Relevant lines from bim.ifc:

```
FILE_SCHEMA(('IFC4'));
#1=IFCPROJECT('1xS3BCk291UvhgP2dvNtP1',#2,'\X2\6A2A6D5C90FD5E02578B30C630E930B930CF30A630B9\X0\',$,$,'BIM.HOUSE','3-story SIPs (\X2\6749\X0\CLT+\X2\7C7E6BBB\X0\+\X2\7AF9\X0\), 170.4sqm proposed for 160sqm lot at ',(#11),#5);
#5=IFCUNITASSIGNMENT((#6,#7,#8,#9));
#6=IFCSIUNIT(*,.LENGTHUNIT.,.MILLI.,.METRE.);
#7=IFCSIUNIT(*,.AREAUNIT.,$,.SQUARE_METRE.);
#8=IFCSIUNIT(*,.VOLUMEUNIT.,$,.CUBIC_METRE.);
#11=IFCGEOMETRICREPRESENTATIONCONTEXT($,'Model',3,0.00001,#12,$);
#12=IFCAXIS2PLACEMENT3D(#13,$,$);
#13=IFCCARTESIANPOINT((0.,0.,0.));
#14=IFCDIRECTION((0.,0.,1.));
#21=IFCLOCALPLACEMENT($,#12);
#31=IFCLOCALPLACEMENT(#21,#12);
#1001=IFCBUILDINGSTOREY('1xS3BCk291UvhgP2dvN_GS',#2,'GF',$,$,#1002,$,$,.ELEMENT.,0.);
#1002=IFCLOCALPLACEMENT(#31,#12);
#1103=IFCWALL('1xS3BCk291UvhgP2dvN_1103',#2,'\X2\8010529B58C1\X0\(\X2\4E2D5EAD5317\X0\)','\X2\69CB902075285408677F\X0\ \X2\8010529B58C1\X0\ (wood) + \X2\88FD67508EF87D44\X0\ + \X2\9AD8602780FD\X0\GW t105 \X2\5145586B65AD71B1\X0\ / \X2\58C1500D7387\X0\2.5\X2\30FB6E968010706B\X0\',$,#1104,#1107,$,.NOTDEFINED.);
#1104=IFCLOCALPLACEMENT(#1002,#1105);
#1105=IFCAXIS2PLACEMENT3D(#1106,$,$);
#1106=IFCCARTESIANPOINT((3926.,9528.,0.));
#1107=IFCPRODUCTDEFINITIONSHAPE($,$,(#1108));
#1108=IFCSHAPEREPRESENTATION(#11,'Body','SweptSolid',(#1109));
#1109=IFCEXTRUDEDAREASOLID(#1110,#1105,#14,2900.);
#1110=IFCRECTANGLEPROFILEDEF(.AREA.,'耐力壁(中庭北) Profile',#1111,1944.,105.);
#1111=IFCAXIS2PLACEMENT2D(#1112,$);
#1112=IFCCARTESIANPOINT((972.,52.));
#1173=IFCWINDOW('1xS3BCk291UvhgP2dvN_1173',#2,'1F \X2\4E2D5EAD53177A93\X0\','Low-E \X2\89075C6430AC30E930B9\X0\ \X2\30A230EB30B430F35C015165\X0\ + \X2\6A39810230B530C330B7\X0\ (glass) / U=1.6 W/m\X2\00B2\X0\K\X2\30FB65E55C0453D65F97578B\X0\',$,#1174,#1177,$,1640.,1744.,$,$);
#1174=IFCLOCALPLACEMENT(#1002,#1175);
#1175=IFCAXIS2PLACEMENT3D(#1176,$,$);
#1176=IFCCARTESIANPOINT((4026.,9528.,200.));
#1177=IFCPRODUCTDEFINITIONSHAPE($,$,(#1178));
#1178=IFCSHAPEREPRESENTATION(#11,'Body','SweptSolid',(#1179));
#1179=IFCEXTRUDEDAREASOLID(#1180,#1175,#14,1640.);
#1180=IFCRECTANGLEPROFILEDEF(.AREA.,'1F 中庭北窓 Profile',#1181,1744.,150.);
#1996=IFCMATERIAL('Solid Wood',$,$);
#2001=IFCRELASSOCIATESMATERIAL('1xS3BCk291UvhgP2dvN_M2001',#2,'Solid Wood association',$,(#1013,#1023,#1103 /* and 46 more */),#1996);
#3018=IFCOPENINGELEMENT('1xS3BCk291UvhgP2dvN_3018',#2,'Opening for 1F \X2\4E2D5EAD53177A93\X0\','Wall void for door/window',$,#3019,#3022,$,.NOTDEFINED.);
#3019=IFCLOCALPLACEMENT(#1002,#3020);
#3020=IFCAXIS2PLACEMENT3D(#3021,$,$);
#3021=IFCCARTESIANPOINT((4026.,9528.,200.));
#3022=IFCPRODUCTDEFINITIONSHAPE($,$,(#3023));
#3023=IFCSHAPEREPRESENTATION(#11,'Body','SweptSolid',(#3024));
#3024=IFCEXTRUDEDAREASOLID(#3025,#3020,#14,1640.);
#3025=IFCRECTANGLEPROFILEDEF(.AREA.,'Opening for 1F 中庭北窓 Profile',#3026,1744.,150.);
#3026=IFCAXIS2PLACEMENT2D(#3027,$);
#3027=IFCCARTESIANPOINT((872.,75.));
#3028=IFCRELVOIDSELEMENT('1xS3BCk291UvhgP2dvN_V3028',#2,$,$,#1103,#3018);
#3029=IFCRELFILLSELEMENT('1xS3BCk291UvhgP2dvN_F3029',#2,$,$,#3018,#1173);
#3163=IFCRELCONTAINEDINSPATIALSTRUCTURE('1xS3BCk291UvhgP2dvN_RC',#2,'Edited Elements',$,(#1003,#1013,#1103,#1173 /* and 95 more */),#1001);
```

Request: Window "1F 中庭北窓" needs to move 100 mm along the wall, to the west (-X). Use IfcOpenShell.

```python
import ifcopenshell
import ifcopenshell.api.geometry
import ifcopenshell.util.placement
import ifcopenshell.util.unit

model = ifcopenshell.open("bim.ifc")
unit_scale = ifcopenshell.util.unit.calculate_unit_scale(model)

window = model.by_guid("1xS3BCk291UvhgP2dvN_1173")
opening = window.FillsVoids[0].RelatingOpeningElement
wall = opening.VoidsElements[0].RelatingBuildingElement

wall_matrix = ifcopenshell.util.placement.get_local_placement(wall.ObjectPlacement)
shift = wall_matrix[:3, 0] * -0.1 / unit_scale
before = ifcopenshell.util.placement.get_local_placement(window.ObjectPlacement)[:3, 3].copy()

# The window is not placed relative to its opening, so move both.
for product in (opening, window):
    matrix = ifcopenshell.util.placement.get_local_placement(product.ObjectPlacement)
    matrix[:3, 3] += shift
    ifcopenshell.api.geometry.edit_object_placement(model, product=product, matrix=matrix, is_si=False)

after = ifcopenshell.util.placement.get_local_placement(window.ObjectPlacement)[:3, 3]
print("window moved by", (after - before).round(3) + 0.0)

model.write("bim_updated.ifc")
```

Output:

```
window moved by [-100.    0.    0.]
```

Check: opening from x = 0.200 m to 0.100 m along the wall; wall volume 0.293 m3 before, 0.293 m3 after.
